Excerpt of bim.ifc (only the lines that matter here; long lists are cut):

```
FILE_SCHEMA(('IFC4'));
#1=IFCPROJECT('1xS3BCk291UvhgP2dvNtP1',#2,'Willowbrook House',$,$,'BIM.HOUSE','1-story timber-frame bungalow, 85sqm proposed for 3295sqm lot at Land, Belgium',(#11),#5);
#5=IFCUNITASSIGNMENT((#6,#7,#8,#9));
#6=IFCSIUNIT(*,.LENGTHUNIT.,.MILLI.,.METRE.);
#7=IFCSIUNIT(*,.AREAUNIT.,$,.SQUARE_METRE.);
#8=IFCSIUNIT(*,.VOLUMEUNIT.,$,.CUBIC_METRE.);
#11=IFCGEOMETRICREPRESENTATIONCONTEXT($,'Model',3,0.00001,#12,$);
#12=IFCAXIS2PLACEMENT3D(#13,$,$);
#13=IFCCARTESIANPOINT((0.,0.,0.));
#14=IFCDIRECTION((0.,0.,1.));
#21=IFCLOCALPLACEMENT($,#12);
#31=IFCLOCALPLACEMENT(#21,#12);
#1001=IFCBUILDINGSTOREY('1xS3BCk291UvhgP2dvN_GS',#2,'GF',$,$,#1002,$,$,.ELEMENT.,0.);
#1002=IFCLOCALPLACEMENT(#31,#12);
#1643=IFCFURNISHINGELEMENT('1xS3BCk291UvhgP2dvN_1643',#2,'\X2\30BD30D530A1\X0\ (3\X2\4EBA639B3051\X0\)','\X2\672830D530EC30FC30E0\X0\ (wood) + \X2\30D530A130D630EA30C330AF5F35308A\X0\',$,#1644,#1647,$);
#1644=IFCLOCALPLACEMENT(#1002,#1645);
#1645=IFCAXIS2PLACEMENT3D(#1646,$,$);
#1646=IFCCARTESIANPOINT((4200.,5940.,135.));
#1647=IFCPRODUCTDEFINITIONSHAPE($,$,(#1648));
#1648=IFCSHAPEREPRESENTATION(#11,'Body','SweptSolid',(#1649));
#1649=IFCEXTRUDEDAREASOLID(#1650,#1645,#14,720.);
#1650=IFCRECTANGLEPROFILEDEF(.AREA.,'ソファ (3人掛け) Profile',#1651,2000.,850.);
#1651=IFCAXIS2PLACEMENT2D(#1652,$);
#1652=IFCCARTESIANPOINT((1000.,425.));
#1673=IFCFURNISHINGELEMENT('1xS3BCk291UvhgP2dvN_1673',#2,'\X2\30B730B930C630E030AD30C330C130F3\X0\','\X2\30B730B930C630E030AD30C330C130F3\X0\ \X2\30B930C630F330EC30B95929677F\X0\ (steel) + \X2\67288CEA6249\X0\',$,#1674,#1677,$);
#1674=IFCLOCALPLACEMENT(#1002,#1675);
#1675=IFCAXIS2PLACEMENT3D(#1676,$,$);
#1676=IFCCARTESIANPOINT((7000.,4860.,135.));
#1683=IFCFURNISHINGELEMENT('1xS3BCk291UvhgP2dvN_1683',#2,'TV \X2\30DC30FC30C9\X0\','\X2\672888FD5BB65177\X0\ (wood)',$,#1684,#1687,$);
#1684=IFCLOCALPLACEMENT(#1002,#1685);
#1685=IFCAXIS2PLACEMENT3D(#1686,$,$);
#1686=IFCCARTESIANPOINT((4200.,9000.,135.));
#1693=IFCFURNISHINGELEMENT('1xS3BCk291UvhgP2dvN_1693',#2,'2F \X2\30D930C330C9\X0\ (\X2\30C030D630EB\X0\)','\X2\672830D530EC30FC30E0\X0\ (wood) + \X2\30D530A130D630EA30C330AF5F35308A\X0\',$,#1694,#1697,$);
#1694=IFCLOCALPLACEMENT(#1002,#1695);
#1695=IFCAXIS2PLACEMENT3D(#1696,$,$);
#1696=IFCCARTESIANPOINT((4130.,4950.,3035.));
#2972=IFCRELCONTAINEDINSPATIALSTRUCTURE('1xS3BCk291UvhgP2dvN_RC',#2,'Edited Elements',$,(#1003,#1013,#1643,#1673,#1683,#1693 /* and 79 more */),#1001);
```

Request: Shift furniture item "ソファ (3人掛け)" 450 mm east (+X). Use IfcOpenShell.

```python
import ifcopenshell
import ifcopenshell.api.geometry
import ifcopenshell.util.placement
import ifcopenshell.util.unit

model = ifcopenshell.open("bim.ifc")
unit_scale = ifcopenshell.util.unit.calculate_unit_scale(model)

item = model.by_id(1643)
matrix = ifcopenshell.util.placement.get_local_placement(item.ObjectPlacement)
matrix[0, 3] += 0.45 / unit_scale
ifcopenshell.api.geometry.edit_object_placement(model, product=item, matrix=matrix, is_si=False)

print(ifcopenshell.util.placement.get_local_placement(item.ObjectPlacement).round(3) + 0.0)

model.write("bim_v2.ifc")
```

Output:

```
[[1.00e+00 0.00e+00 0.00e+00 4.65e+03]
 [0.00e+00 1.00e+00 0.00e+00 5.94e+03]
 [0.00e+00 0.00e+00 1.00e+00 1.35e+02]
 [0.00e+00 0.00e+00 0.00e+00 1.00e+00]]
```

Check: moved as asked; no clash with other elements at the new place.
